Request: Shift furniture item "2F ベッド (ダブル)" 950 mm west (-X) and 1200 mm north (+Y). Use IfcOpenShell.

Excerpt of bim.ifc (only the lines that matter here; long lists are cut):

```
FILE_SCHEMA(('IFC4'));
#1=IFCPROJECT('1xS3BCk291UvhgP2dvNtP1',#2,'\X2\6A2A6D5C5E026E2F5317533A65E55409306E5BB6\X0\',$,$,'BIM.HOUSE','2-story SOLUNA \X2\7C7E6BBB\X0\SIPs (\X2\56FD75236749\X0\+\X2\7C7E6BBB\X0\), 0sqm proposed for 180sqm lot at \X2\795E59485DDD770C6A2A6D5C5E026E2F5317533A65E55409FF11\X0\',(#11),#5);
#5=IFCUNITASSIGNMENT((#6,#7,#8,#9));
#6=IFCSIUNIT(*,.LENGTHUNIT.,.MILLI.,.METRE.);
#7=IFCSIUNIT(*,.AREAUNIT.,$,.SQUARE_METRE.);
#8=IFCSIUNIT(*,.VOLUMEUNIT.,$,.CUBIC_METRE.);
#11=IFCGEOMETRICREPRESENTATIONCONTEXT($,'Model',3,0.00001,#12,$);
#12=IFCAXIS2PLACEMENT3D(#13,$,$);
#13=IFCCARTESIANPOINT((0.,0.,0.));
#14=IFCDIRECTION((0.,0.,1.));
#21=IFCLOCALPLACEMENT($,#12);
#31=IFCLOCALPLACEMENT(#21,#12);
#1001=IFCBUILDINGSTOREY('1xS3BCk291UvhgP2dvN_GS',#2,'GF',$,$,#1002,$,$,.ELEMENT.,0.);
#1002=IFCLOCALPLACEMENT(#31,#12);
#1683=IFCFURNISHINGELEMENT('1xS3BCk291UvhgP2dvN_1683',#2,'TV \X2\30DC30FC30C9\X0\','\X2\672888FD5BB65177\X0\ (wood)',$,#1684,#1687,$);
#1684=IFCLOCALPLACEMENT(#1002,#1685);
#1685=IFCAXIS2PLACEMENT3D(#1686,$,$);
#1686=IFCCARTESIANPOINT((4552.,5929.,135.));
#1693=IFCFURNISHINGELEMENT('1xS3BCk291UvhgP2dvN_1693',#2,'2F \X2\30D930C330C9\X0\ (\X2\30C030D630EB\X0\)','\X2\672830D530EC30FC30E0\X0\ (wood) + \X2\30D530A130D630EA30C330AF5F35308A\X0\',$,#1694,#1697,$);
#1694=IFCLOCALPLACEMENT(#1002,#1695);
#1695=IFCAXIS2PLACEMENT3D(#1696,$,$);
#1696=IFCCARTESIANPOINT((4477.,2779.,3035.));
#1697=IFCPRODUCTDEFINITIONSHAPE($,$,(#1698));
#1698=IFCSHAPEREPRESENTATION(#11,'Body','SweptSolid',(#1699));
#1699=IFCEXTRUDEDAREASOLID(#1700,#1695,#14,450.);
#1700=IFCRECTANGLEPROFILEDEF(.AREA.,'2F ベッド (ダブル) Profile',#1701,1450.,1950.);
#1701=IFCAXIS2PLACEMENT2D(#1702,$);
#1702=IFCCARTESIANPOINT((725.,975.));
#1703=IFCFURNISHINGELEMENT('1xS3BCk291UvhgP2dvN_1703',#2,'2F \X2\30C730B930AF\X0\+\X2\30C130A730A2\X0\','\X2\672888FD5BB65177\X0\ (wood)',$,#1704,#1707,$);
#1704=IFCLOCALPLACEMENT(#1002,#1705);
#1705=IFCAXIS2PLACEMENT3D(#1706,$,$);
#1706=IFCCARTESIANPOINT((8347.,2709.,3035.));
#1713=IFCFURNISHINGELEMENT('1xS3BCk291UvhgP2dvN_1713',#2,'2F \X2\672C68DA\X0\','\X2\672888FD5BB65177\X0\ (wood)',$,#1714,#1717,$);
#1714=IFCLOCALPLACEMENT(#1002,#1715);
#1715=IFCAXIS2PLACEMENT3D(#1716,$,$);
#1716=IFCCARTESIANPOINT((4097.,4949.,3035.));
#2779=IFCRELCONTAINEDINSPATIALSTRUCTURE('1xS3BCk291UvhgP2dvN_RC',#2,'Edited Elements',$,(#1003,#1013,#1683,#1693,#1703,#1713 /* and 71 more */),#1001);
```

```python
import ifcopenshell
import ifcopenshell.api.geometry
import ifcopenshell.util.placement

model = ifcopenshell.open("bim.ifc")

item = model.by_id(1693)
matrix = ifcopenshell.util.placement.get_local_placement(item.ObjectPlacement)
matrix[0, 3] -= 950.0
matrix[1, 3] += 1200.0
ifcopenshell.api.geometry.edit_object_placement(model, product=item, matrix=matrix, is_si=False)

print(ifcopenshell.util.placement.get_local_placement(item.ObjectPlacement).round(3) + 0.0)

model.write("bim_rev.ifc")
```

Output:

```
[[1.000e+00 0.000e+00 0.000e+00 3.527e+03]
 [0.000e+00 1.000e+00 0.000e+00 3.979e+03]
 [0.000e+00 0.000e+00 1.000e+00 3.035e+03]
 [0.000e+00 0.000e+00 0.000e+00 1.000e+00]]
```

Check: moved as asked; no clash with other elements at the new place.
